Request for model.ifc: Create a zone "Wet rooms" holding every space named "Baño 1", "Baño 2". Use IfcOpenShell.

First a look at what the model holds.

```python
import ifcopenshell

model = ifcopenshell.open("model.ifc")
print(model.schema)
seen = {}
for space in model.by_type("IfcSpace"):
    seen[space.LongName] = seen.get(space.LongName, 0) + 1
for name, count in sorted(seen.items(), key=str):
    print(count, "x", name)
print("zones:", [z.Name for z in model.by_type("IfcZone")][:20])
```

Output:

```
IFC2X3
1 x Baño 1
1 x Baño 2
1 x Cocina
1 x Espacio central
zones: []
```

```python
import ifcopenshell
import ifcopenshell.api.group
import ifcopenshell.api.root

model = ifcopenshell.open("model.ifc")

names = {"Baño 1", "Baño 2"}
spaces = [s for s in model.by_type("IfcSpace") if s.LongName in names]

zone = ifcopenshell.api.root.create_entity(model, ifc_class="IfcZone", name="Wet rooms")
ifcopenshell.api.group.assign_group(model, products=spaces, group=zone)
print(len(spaces), "spaces in", zone.Name)

model.write("model-out.ifc")
```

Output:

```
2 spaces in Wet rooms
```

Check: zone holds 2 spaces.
